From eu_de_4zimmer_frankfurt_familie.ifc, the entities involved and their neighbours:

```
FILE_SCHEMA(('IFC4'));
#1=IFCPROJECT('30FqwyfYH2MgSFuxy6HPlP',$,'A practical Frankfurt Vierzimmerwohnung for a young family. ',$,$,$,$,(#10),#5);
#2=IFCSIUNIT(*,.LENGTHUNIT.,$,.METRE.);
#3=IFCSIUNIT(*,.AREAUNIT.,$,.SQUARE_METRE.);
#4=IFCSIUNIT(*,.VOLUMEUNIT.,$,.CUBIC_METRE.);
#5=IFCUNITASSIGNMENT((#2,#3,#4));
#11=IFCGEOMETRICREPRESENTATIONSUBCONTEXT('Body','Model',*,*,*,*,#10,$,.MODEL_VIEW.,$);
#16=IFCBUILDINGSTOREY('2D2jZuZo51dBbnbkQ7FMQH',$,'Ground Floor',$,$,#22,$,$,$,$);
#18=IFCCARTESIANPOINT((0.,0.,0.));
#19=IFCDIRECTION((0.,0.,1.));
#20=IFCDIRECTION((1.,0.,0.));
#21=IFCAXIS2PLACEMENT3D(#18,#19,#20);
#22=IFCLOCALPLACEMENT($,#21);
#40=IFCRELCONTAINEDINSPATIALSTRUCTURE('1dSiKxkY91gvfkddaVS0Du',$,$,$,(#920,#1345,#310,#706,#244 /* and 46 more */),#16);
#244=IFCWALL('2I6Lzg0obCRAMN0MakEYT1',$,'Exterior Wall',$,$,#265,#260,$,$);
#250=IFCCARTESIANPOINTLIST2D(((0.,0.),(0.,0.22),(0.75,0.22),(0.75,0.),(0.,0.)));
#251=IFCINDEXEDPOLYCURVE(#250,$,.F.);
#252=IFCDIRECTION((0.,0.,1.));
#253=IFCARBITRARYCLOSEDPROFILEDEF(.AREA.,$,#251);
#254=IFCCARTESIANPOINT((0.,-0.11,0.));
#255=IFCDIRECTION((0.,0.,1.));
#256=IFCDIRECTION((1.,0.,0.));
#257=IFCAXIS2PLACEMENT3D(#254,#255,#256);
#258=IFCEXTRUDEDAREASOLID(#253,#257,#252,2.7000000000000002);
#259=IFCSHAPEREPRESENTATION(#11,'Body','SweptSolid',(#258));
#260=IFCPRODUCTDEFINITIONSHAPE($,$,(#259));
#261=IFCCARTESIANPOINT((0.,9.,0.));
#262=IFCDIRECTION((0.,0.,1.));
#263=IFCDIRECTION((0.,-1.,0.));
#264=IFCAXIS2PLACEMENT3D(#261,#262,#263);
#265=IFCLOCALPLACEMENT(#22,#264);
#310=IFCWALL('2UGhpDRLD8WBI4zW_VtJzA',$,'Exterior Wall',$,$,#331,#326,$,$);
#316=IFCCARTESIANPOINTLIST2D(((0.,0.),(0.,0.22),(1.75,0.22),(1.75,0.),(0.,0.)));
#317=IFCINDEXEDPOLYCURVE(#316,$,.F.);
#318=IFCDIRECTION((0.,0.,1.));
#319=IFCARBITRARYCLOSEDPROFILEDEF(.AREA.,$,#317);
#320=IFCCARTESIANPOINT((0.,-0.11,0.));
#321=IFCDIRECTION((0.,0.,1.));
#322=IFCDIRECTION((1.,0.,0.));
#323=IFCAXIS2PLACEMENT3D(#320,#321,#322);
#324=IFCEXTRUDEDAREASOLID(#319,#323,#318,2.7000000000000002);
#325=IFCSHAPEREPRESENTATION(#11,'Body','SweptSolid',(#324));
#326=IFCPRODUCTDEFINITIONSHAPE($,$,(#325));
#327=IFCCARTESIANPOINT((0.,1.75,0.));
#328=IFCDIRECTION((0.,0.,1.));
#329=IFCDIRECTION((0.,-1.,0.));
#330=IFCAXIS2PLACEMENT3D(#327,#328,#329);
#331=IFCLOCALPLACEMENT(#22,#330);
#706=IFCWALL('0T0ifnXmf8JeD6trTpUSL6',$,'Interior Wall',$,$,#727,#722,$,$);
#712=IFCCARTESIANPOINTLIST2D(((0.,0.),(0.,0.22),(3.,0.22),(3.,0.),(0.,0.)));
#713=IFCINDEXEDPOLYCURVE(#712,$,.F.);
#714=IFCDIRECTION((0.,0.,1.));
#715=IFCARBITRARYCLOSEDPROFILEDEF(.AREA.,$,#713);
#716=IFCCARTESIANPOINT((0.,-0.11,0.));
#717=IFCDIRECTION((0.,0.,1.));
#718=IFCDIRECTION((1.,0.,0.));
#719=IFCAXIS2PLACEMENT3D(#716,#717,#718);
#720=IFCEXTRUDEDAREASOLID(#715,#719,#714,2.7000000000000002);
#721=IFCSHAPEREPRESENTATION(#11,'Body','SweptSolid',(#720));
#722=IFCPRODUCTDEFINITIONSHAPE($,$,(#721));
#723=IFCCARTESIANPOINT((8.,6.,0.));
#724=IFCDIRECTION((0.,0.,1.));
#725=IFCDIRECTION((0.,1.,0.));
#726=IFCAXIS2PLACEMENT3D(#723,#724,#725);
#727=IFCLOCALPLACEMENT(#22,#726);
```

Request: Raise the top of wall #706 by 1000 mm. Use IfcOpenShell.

```python
import ifcopenshell
import ifcopenshell.geom
import ifcopenshell.util.representation
import ifcopenshell.util.shape

model = ifcopenshell.open("eu_de_4zimmer_frankfurt_familie.ifc")
settings = ifcopenshell.geom.settings()


def volume(element):
    """Net volume in cubic metres, openings subtracted."""
    shape = ifcopenshell.geom.create_shape(settings, element)
    return ifcopenshell.util.shape.get_volume(shape.geometry)


wall = model.by_id(706)
before = volume(wall)

body = ifcopenshell.util.representation.get_representation(wall, "Model", "Body")
solid = body.Items[0]
old_height = solid.Depth
solid.Depth += 1.0
after = volume(wall)

print(f"height {old_height:g} -> {solid.Depth:g}, volume {before:.3f} -> {after:.3f} m3")

model.write("eu_de_4zimmer_frankfurt_familie_updated.ifc")
```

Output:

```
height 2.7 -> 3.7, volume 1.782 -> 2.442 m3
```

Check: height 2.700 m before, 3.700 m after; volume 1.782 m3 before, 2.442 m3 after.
